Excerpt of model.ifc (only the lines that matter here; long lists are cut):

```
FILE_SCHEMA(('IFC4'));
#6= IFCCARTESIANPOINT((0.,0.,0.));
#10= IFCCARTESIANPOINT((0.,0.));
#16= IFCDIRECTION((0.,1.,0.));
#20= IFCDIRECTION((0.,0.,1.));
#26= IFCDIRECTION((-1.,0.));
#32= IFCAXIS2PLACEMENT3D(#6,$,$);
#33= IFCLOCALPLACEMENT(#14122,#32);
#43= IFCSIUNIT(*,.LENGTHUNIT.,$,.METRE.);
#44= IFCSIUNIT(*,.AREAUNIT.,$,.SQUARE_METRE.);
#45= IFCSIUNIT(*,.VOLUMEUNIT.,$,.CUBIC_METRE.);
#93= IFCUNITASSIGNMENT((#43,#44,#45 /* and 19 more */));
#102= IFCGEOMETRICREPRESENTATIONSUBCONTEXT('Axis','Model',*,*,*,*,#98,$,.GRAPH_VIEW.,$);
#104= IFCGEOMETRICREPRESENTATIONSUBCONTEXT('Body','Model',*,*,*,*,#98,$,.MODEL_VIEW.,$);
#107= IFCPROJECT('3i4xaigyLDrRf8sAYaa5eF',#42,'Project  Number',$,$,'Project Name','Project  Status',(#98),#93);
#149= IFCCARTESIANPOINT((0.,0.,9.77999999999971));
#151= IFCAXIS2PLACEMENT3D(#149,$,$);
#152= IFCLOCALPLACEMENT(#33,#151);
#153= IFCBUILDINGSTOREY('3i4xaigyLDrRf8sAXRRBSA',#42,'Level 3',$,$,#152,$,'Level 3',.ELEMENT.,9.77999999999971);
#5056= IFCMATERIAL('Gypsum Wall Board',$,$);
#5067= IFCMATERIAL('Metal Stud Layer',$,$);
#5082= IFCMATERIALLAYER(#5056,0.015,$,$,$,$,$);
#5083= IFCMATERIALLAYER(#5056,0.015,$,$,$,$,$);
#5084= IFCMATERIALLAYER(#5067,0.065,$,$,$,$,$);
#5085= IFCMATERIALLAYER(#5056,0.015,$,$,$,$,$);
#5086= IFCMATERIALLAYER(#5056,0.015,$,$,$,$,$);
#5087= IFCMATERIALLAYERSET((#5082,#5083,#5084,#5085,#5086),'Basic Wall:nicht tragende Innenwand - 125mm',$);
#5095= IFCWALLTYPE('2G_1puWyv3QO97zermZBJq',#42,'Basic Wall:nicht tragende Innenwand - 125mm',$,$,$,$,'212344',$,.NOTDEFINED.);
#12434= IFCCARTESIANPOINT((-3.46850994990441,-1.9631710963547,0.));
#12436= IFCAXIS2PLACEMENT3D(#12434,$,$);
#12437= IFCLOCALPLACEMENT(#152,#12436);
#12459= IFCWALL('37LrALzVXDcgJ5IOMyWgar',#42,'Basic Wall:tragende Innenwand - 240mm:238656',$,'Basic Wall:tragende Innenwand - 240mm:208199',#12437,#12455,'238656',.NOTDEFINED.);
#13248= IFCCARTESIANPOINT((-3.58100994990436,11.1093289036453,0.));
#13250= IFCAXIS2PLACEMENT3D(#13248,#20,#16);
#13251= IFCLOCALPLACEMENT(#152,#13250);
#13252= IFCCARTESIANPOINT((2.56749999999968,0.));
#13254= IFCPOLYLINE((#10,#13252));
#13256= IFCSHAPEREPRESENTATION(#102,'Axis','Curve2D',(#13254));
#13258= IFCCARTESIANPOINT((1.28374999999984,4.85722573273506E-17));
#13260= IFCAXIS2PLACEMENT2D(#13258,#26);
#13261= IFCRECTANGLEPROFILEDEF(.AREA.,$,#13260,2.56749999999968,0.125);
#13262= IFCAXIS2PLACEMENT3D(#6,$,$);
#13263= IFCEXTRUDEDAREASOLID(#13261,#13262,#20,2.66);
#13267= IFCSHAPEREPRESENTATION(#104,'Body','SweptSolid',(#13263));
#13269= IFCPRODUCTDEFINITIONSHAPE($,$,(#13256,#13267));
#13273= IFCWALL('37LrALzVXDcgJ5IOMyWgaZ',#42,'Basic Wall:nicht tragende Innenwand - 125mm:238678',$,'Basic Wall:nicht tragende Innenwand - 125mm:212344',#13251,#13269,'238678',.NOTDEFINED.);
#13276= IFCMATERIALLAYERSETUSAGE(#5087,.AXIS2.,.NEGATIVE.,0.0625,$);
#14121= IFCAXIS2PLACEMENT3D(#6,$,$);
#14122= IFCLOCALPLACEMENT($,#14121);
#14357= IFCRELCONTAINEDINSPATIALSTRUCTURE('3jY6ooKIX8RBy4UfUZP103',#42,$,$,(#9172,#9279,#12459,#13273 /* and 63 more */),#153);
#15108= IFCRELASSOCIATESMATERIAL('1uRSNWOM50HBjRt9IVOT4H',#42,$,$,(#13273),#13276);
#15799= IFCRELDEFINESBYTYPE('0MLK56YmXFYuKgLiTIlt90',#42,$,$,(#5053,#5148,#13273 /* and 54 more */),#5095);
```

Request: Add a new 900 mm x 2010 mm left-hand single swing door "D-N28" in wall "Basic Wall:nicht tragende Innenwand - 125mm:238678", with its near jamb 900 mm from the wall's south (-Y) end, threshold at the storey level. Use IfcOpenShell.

```python
import numpy as np
import ifcopenshell
import ifcopenshell.api.feature
import ifcopenshell.api.geometry
import ifcopenshell.api.root
import ifcopenshell.api.spatial
import ifcopenshell.geom
import ifcopenshell.util.element
import ifcopenshell.util.placement
import ifcopenshell.util.representation
import ifcopenshell.util.shape
import ifcopenshell.util.unit

model = ifcopenshell.open("model.ifc")
unit_scale = ifcopenshell.util.unit.calculate_unit_scale(model)
settings = ifcopenshell.geom.settings()


def volume(element):
    """Net volume in cubic metres, openings subtracted."""
    shape = ifcopenshell.geom.create_shape(settings, element)
    return ifcopenshell.util.shape.get_volume(shape.geometry)


wall = model.by_guid("37LrALzVXDcgJ5IOMyWgaZ")
storey = ifcopenshell.util.element.get_container(wall, ifc_class="IfcBuildingStorey")
context = ifcopenshell.util.representation.get_context(model, "Model", "Body", "MODEL_VIEW")
before = volume(wall)

width, height, from_end, sill = 0.9, 2.01, 0.9, 0.0  # metres

# The wall runs along its own X axis, and the end named is its -X end.
wall_shape = ifcopenshell.geom.create_shape(settings, wall)
x, y, z = ifcopenshell.util.shape.get_vertices(wall_shape.geometry).T
start = x.min() + from_end
face, thickness = float(y.min()), float(y.max() - y.min())
wall_matrix = ifcopenshell.util.placement.get_local_placement(wall.ObjectPlacement)
level = ifcopenshell.util.placement.get_local_placement(storey.ObjectPlacement)[2, 3]


def in_wall(x, y):
    """Placement at x, y metres in the wall's axes, at sill height."""
    matrix = wall_matrix.copy()
    matrix[:, 3] = wall_matrix @ np.array([x / unit_scale, y / unit_scale, 0.0, 1.0])
    matrix[2, 3] = level + sill / unit_scale
    return matrix


# Opening: a box that overshoots both wall faces by 50 mm.
opening = ifcopenshell.api.root.create_entity(model, ifc_class="IfcOpeningElement", predefined_type="OPENING")
box = ifcopenshell.api.geometry.add_wall_representation(
    model, context=context, length=width, height=height, thickness=thickness + 0.1
)
ifcopenshell.api.geometry.assign_representation(model, product=opening, representation=box)
ifcopenshell.api.geometry.edit_object_placement(model, product=opening, matrix=in_wall(start, face - 0.05), is_si=False)
ifcopenshell.api.feature.add_feature(model, feature=opening, element=wall)

door = ifcopenshell.api.root.create_entity(model, ifc_class="IfcDoor", name="D-N28", predefined_type="DOOR")
door.OverallWidth, door.OverallHeight = width / unit_scale, height / unit_scale
door.OperationType = "SINGLE_SWING_LEFT"
body = ifcopenshell.api.geometry.add_door_representation(
    model,
    context=context,
    overall_width=door.OverallWidth,
    overall_height=door.OverallHeight,
    operation_type="SINGLE_SWING_LEFT",
    lining_properties={"LiningDepth": thickness / unit_scale, "ThresholdDepth": thickness / unit_scale},
)
ifcopenshell.api.geometry.assign_representation(model, product=door, representation=body)
ifcopenshell.api.spatial.assign_container(model, products=[door], relating_structure=storey)
ifcopenshell.api.feature.add_filling(model, opening=opening, element=door)

# The lining spans the wall, so the door starts at the wall face.
ifcopenshell.api.geometry.edit_object_placement(model, product=door, matrix=in_wall(start, face), is_si=False)

after = volume(wall)

print(f"wall volume {before:.3f} -> {after:.3f} m3")

model.write("model_v2.ifc")
```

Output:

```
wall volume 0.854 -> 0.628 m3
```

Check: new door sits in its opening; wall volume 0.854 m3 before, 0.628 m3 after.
